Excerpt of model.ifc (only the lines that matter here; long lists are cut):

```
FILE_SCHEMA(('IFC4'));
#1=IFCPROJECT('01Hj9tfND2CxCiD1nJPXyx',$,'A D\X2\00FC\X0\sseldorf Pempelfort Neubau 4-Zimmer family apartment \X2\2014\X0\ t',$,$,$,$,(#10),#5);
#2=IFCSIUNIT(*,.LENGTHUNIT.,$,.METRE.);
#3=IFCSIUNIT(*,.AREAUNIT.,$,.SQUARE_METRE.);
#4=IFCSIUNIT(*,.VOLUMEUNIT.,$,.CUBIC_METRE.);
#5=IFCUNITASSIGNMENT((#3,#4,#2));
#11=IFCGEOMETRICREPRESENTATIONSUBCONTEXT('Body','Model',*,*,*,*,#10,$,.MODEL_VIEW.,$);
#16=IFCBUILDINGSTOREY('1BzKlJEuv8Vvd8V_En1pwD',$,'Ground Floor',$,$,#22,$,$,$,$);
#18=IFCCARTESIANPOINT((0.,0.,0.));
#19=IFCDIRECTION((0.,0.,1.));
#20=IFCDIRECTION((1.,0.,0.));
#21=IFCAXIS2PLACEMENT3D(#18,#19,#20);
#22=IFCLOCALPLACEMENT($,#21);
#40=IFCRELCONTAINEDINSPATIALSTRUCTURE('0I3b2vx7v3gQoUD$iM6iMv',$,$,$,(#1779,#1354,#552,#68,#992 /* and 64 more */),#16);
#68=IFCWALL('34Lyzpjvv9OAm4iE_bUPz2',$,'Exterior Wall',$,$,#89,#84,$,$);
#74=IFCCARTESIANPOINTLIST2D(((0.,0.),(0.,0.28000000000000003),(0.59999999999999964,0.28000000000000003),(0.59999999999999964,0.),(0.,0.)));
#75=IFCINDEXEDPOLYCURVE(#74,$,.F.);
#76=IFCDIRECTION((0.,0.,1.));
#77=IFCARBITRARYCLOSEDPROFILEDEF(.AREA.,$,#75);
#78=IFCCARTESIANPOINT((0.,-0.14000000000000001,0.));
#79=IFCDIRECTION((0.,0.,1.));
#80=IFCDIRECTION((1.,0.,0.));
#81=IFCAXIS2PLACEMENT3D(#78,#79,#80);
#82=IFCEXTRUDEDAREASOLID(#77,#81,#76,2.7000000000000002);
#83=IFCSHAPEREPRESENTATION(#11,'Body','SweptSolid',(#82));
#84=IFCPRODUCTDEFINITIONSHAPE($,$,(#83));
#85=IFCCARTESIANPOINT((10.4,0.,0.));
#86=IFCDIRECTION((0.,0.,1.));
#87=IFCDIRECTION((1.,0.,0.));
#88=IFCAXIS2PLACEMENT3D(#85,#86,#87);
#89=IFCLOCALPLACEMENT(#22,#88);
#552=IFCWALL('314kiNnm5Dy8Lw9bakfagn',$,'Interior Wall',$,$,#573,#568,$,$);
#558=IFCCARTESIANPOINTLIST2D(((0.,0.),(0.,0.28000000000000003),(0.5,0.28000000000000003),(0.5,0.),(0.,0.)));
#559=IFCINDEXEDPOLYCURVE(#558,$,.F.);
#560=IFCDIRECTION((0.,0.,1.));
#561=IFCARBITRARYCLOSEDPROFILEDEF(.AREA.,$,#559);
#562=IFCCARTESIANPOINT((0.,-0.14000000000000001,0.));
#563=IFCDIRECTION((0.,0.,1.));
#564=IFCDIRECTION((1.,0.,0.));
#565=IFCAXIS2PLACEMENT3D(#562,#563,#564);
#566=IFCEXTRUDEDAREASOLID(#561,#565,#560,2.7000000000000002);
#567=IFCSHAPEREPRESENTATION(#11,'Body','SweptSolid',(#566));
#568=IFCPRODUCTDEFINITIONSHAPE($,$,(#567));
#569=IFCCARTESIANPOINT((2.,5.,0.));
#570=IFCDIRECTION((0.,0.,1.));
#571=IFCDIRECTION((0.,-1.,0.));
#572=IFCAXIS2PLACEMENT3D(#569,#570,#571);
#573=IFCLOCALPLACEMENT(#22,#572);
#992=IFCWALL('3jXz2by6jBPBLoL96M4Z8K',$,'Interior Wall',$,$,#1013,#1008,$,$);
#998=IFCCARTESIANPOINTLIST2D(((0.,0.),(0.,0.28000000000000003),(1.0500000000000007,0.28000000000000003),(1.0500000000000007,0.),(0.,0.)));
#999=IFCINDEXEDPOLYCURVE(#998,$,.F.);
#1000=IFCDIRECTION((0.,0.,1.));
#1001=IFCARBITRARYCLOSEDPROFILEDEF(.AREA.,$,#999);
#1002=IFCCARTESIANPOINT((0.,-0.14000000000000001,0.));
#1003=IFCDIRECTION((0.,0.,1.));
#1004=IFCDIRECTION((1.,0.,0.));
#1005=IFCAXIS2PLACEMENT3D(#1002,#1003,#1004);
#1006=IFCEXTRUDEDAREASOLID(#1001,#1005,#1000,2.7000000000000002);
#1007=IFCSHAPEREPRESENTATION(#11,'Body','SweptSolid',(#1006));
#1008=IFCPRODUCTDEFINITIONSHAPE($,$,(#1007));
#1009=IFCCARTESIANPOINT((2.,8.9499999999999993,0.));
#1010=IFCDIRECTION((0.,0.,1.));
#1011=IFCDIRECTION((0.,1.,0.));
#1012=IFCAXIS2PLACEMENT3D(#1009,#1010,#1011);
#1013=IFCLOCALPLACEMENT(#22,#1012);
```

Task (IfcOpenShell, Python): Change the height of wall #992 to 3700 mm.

```python
import ifcopenshell
import ifcopenshell.geom
import ifcopenshell.util.representation
import ifcopenshell.util.shape

model = ifcopenshell.open("model.ifc")
settings = ifcopenshell.geom.settings()


def volume(element):
    """Net volume in cubic metres, openings subtracted."""
    shape = ifcopenshell.geom.create_shape(settings, element)
    return ifcopenshell.util.shape.get_volume(shape.geometry)


wall = model.by_id(992)
before = volume(wall)

body = ifcopenshell.util.representation.get_representation(wall, "Model", "Body")
solid = body.Items[0]
old_height = solid.Depth
solid.Depth = 3.7
after = volume(wall)

print(f"height {old_height:g} -> {solid.Depth:g}, volume {before:.3f} -> {after:.3f} m3")

model.write("model_rev.ifc")
```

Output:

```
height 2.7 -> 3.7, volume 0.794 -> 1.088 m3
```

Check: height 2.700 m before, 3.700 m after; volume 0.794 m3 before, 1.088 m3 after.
